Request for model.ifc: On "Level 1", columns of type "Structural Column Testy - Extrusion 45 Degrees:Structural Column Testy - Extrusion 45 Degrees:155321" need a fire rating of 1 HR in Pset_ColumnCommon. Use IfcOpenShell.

First a look at what the model holds.

```python
import ifcopenshell
import ifcopenshell.util.element

model = ifcopenshell.open("model.ifc")
print(model.schema)
storey = next(s for s in model.by_type("IfcBuildingStorey") if s.Name == "Level 1")
columns = [e for e in ifcopenshell.util.element.get_decomposition(storey) if e.is_a("IfcColumn")]
seen = {}
for e in columns:
    element_type = ifcopenshell.util.element.get_type(e)
    key = (element_type.Name if element_type != e and element_type else None, ifcopenshell.util.element.get_pset(e, "Pset_ColumnCommon", "FireRating"))
    seen[key] = seen.get(key, 0) + 1
for (name, value), count in sorted(seen.items(), key=str):
    print(count, "x", name, "|", value)
```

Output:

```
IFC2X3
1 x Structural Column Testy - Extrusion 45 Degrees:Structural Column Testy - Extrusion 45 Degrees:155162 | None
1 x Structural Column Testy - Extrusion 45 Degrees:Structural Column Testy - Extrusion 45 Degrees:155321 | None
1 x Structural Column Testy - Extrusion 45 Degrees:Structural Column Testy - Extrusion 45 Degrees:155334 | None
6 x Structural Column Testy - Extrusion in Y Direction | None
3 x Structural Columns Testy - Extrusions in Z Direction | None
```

```python
import ifcopenshell
import ifcopenshell.api.pset
import ifcopenshell.util.element

model = ifcopenshell.open("model.ifc")

storey = next(s for s in model.by_type("IfcBuildingStorey") if s.Name == "Level 1")
columns = [e for e in ifcopenshell.util.element.get_decomposition(storey) if e.is_a("IfcColumn")]

count = 0
for e in columns:
    element_type = ifcopenshell.util.element.get_type(e)
    if element_type in (None, e) or element_type.Name != "Structural Column Testy - Extrusion 45 Degrees:Structural Column Testy - Extrusion 45 Degrees:155321":
        continue
    # add_pset returns the element's existing set when there is one.
    pset = ifcopenshell.api.pset.add_pset(model, product=e, name="Pset_ColumnCommon")
    ifcopenshell.api.pset.edit_pset(model, pset=pset, properties={"FireRating": "1 HR"})
    count += 1

print(count, "columns updated")

model.write("model_v2.ifc")
```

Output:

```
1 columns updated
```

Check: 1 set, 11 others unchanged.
